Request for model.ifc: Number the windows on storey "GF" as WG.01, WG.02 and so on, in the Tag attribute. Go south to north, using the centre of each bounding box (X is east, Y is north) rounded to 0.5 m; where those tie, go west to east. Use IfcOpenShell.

First a look at what the model holds.

```python
import ifcopenshell
import ifcopenshell.util.element
import ifcopenshell.util.placement

model = ifcopenshell.open("model.ifc")
print(model.schema)
storey = next(s for s in model.by_type("IfcBuildingStorey") if s.Name == "GF")
windows = [e for e in ifcopenshell.util.element.get_decomposition(storey) if e.is_a("IfcWindow")]
for e in sorted(windows, key=lambda e: e.id()):
    origin = ifcopenshell.util.placement.get_local_placement(e.ObjectPlacement)[:3, 3]
    print(e.id(), e.Tag, e.Name, origin.round(2) + 0.0, sep=" | ")
```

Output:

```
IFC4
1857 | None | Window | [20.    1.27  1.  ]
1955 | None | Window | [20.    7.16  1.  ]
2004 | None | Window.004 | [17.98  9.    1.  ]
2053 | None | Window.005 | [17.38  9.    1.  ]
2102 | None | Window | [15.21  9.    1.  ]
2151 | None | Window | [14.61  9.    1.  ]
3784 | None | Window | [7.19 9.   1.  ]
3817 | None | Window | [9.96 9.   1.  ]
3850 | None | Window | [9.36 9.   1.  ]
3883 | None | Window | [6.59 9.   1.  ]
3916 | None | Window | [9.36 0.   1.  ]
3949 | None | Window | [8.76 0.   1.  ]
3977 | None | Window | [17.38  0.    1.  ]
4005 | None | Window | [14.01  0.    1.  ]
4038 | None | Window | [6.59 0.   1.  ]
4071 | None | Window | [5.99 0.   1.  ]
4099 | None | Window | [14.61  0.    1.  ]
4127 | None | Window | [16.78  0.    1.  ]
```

```python
import ifcopenshell
import ifcopenshell.geom
import ifcopenshell.util.element
import ifcopenshell.util.shape

model = ifcopenshell.open("model.ifc")
settings = ifcopenshell.geom.settings()
settings.set("use-world-coords", True)


def centre(element):
    shape = ifcopenshell.geom.create_shape(settings, element)
    return ifcopenshell.util.shape.get_bbox_centroid(shape.geometry)


storey = next(s for s in model.by_type("IfcBuildingStorey") if s.Name == "GF")
windows = [e for e in ifcopenshell.util.element.get_decomposition(storey) if e.is_a("IfcWindow")]

# Insertion points can sit at a corner or the storey origin, so sort by the geometry (in metres).
centres = {e: centre(e) for e in windows}
windows.sort(key=lambda e: (round(centres[e][1] / 0.5), centres[e][0]))

for i, e in enumerate(windows, start=1):
    number = f"WG.{i:02d}"
    e.Tag = number
    print(e.id(), number)

model.write("model_edited.ifc")
```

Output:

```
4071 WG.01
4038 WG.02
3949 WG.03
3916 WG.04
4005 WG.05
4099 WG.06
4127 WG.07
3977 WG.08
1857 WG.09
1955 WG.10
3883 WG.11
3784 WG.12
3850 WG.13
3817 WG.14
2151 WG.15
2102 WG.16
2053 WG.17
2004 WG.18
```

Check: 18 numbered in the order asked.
